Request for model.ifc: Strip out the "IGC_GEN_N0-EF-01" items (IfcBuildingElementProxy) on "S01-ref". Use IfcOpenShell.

First a look at what the model holds.

```python
import ifcopenshell
import ifcopenshell.util.element

model = ifcopenshell.open("model.ifc")
print(model.schema)
storey = next(s for s in model.by_type("IfcBuildingStorey") if s.Name == "S01-ref")
proxies = [e for e in ifcopenshell.util.element.get_decomposition(storey) if e.is_a("IfcBuildingElementProxy")]
seen = {}
for e in proxies:
    element_type = ifcopenshell.util.element.get_type(e)
    name = element_type.Name if element_type not in (None, e) else None
    seen[name] = seen.get(name, 0) + 1
for name, count in sorted(seen.items(), key=str):
    print(count, "x", name)
```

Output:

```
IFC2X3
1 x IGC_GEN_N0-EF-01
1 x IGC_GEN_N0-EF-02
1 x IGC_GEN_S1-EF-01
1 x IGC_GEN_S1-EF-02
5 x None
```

```python
import ifcopenshell
import ifcopenshell.api.root
import ifcopenshell.util.element

model = ifcopenshell.open("model.ifc")

storey = next(s for s in model.by_type("IfcBuildingStorey") if s.Name == "S01-ref")
proxies = [e for e in ifcopenshell.util.element.get_decomposition(storey) if e.is_a("IfcBuildingElementProxy")]
targets = [e for e in proxies if (t := ifcopenshell.util.element.get_type(e)) not in (None, e) and t.Name == "IGC_GEN_N0-EF-01"]

for e in targets:
    ifcopenshell.api.root.remove_product(model, product=e)
print(len(targets), "removed")

model.write("model-out.ifc")
```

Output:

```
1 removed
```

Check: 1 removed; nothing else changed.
